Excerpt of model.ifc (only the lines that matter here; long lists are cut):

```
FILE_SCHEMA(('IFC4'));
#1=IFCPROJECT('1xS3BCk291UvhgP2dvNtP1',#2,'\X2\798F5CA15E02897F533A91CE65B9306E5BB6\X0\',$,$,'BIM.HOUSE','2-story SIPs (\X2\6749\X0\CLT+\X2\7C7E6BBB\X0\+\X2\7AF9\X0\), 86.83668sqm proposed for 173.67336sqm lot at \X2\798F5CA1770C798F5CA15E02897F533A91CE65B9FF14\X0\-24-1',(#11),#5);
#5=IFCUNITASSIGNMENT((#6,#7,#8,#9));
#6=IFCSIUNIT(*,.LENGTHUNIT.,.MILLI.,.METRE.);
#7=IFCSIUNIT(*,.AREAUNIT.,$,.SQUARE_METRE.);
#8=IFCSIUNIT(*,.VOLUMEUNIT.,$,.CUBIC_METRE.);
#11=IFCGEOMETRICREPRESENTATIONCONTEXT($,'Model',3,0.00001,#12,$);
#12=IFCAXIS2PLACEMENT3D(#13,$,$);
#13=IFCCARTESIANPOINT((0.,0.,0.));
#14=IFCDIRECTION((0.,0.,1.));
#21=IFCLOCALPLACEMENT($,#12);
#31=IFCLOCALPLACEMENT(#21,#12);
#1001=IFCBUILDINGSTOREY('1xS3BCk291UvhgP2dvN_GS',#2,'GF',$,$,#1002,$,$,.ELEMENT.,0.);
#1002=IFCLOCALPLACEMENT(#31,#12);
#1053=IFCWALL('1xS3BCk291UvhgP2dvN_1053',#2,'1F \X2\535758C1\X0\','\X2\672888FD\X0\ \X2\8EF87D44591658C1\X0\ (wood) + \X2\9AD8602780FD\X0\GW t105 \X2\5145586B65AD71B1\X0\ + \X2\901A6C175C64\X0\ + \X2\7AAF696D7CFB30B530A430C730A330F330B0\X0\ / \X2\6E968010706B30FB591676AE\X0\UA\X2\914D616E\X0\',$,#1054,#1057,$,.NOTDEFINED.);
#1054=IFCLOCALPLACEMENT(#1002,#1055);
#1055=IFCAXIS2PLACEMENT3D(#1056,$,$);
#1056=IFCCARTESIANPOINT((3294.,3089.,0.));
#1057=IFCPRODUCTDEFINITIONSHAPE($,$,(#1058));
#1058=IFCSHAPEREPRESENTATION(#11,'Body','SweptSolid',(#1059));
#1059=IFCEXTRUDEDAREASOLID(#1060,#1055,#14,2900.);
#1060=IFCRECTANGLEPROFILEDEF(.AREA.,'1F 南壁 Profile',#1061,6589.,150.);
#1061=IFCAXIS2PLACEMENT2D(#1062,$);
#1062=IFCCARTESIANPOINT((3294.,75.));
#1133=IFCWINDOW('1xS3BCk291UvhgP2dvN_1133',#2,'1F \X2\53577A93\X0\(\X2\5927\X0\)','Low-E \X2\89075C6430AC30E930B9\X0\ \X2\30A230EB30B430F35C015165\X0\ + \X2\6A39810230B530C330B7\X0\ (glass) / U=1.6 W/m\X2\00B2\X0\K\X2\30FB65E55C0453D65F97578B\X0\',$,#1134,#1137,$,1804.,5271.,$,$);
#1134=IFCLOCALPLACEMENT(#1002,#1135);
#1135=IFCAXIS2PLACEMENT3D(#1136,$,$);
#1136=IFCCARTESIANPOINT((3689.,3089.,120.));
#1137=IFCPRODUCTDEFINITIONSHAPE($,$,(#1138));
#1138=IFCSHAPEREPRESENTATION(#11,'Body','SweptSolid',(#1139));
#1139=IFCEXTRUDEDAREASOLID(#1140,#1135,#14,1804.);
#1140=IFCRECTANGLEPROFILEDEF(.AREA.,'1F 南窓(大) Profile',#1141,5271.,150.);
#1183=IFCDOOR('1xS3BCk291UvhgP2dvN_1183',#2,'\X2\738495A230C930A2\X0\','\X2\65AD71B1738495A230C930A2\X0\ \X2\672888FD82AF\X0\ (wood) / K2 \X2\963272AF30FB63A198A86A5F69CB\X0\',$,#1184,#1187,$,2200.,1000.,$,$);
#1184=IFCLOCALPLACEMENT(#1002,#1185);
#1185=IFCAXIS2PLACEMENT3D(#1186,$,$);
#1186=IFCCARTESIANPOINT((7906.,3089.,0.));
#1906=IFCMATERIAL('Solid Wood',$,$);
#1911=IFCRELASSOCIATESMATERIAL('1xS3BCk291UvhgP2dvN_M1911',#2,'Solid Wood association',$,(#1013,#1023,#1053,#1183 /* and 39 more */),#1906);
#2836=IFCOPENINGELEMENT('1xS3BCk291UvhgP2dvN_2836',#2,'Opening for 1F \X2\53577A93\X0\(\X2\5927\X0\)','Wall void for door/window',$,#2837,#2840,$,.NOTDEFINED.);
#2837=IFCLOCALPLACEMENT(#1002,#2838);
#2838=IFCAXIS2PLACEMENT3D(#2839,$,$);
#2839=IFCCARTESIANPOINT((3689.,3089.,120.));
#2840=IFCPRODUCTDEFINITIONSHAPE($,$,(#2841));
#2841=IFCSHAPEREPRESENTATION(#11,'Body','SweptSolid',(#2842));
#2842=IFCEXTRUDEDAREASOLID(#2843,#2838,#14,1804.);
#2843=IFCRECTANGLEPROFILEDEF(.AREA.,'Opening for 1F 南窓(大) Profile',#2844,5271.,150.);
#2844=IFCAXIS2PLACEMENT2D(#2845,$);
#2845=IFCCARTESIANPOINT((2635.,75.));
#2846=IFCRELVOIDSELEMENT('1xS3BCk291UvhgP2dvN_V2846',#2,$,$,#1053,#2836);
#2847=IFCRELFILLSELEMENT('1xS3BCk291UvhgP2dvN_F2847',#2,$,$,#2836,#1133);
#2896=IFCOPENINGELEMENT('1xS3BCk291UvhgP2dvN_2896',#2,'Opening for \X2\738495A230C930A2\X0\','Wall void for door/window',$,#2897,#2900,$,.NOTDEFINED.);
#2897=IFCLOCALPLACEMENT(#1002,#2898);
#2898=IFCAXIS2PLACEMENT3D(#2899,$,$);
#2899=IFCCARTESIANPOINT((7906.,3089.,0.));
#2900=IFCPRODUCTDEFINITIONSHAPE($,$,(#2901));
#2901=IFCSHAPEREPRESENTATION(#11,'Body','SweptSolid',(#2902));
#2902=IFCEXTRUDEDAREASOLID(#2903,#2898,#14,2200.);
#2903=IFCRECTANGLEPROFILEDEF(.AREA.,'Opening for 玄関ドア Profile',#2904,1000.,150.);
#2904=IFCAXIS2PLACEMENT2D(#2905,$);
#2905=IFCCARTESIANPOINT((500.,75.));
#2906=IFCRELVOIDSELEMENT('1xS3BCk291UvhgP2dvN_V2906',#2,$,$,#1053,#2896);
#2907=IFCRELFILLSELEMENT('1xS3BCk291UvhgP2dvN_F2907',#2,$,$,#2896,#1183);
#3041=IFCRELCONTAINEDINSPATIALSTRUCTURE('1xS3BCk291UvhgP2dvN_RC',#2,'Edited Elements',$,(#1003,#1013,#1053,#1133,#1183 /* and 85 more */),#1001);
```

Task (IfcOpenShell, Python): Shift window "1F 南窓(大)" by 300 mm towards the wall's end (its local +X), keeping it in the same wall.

```python
import ifcopenshell
import ifcopenshell.api.geometry
import ifcopenshell.util.placement
import ifcopenshell.util.unit

model = ifcopenshell.open("model.ifc")
unit_scale = ifcopenshell.util.unit.calculate_unit_scale(model)

window = model.by_id(1133)
opening = window.FillsVoids[0].RelatingOpeningElement
wall = opening.VoidsElements[0].RelatingBuildingElement

wall_matrix = ifcopenshell.util.placement.get_local_placement(wall.ObjectPlacement)
shift = wall_matrix[:3, 0] * 0.3 / unit_scale
before = ifcopenshell.util.placement.get_local_placement(window.ObjectPlacement)[:3, 3].copy()

# The window is not placed relative to its opening, so move both.
for product in (opening, window):
    matrix = ifcopenshell.util.placement.get_local_placement(product.ObjectPlacement)
    matrix[:3, 3] += shift
    ifcopenshell.api.geometry.edit_object_placement(model, product=product, matrix=matrix, is_si=False)

after = ifcopenshell.util.placement.get_local_placement(window.ObjectPlacement)[:3, 3]
print("window moved by", (after - before).round(3) + 0.0)

model.write("model_v2.ifc")
```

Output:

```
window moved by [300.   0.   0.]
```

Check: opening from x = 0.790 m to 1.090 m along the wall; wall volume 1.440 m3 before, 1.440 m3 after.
